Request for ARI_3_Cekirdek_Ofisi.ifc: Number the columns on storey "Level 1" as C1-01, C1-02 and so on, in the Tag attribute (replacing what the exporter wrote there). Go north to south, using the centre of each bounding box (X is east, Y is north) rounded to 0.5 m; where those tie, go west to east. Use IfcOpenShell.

First a look at what the model holds.

```python
import ifcopenshell
import ifcopenshell.util.element
import ifcopenshell.util.placement

model = ifcopenshell.open("ARI_3_Cekirdek_Ofisi.ifc")
print(model.schema)
storey = next(s for s in model.by_type("IfcBuildingStorey") if s.Name == "Level 1")
columns = [e for e in ifcopenshell.util.element.get_decomposition(storey) if e.is_a("IfcColumn")]
for e in sorted(columns, key=lambda e: e.id()):
    origin = ifcopenshell.util.placement.get_local_placement(e.ObjectPlacement)[:3, 3]
    print(e.id(), e.Tag, e.Name, origin.round(2) + 0.0, sep=" | ")
```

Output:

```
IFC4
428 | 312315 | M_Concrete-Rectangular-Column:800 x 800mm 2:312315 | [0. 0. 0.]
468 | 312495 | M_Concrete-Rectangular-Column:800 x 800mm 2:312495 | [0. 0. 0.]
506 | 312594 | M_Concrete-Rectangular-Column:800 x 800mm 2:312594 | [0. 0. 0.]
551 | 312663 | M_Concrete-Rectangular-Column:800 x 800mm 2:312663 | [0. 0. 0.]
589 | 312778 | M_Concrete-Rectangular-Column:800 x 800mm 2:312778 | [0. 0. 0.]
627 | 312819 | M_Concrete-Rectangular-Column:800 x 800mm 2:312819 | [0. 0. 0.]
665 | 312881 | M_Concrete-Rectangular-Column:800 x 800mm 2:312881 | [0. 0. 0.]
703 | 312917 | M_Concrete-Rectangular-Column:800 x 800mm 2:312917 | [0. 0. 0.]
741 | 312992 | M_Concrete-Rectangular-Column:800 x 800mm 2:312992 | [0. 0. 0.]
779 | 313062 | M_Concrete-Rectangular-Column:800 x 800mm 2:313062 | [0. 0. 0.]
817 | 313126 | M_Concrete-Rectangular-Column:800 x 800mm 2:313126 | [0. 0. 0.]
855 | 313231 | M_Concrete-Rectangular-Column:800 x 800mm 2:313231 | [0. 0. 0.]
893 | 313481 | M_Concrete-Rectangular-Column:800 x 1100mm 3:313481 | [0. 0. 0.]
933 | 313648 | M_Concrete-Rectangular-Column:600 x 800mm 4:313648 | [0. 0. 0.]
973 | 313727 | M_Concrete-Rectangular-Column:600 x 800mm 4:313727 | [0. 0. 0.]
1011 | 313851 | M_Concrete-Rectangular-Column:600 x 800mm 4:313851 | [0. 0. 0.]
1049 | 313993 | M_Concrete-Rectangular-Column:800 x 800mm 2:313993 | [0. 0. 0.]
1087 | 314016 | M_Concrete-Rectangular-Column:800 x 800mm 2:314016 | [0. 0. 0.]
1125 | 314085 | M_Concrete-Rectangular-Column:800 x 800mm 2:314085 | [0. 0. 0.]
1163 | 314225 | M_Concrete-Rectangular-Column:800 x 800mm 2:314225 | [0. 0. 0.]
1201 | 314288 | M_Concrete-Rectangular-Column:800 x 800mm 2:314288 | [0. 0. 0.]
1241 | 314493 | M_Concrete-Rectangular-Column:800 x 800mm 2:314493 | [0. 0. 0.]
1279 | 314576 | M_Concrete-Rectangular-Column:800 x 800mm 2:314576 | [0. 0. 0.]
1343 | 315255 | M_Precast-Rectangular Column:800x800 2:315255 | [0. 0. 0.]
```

```python
import ifcopenshell
import ifcopenshell.geom
import ifcopenshell.util.element
import ifcopenshell.util.shape

model = ifcopenshell.open("ARI_3_Cekirdek_Ofisi.ifc")
settings = ifcopenshell.geom.settings()
settings.set("use-world-coords", True)


def centre(element):
    shape = ifcopenshell.geom.create_shape(settings, element)
    return ifcopenshell.util.shape.get_bbox_centroid(shape.geometry)


storey = next(s for s in model.by_type("IfcBuildingStorey") if s.Name == "Level 1")
columns = [e for e in ifcopenshell.util.element.get_decomposition(storey) if e.is_a("IfcColumn")]

# Insertion points can sit at a corner or the storey origin, so sort by the geometry (in metres).
centres = {e: centre(e) for e in columns}
columns.sort(key=lambda e: (-round(centres[e][1] / 0.5), centres[e][0]))

for i, e in enumerate(columns, start=1):
    number = f"C1-{i:02d}"
    e.Tag = number
    print(e.id(), number)

model.write("ARI_3_Cekirdek_Ofisi_edited.ifc")
```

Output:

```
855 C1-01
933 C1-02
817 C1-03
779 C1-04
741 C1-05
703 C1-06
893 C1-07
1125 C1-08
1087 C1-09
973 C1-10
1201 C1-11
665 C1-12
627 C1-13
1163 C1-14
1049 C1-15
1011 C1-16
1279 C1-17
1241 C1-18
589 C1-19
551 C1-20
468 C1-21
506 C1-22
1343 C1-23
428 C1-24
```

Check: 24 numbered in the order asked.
